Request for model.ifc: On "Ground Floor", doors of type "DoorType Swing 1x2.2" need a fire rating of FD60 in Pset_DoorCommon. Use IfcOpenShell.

First a look at what the model holds.

```python
import ifcopenshell
import ifcopenshell.util.element

model = ifcopenshell.open("model.ifc")
print(model.schema)
storey = next(s for s in model.by_type("IfcBuildingStorey") if s.Name == "Ground Floor")
doors = [e for e in ifcopenshell.util.element.get_decomposition(storey) if e.is_a("IfcDoor")]
seen = {}
for e in doors:
    element_type = ifcopenshell.util.element.get_type(e)
    key = (element_type.Name if element_type != e and element_type else None, ifcopenshell.util.element.get_pset(e, "Pset_DoorCommon", "FireRating"))
    seen[key] = seen.get(key, 0) + 1
for (name, value), count in sorted(seen.items(), key=str):
    print(count, "x", name, "|", value)
```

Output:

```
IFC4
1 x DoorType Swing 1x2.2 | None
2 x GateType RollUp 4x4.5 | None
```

```python
import ifcopenshell
import ifcopenshell.api.pset
import ifcopenshell.util.element

model = ifcopenshell.open("model.ifc")

storey = next(s for s in model.by_type("IfcBuildingStorey") if s.Name == "Ground Floor")
doors = [e for e in ifcopenshell.util.element.get_decomposition(storey) if e.is_a("IfcDoor")]

count = 0
for e in doors:
    element_type = ifcopenshell.util.element.get_type(e)
    if element_type in (None, e) or element_type.Name != "DoorType Swing 1x2.2":
        continue
    # add_pset returns the element's existing set when there is one.
    pset = ifcopenshell.api.pset.add_pset(model, product=e, name="Pset_DoorCommon")
    ifcopenshell.api.pset.edit_pset(model, pset=pset, properties={"FireRating": "FD60"})
    count += 1

print(count, "doors updated")

model.write("model_updated.ifc")
```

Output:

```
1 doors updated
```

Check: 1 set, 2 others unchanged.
